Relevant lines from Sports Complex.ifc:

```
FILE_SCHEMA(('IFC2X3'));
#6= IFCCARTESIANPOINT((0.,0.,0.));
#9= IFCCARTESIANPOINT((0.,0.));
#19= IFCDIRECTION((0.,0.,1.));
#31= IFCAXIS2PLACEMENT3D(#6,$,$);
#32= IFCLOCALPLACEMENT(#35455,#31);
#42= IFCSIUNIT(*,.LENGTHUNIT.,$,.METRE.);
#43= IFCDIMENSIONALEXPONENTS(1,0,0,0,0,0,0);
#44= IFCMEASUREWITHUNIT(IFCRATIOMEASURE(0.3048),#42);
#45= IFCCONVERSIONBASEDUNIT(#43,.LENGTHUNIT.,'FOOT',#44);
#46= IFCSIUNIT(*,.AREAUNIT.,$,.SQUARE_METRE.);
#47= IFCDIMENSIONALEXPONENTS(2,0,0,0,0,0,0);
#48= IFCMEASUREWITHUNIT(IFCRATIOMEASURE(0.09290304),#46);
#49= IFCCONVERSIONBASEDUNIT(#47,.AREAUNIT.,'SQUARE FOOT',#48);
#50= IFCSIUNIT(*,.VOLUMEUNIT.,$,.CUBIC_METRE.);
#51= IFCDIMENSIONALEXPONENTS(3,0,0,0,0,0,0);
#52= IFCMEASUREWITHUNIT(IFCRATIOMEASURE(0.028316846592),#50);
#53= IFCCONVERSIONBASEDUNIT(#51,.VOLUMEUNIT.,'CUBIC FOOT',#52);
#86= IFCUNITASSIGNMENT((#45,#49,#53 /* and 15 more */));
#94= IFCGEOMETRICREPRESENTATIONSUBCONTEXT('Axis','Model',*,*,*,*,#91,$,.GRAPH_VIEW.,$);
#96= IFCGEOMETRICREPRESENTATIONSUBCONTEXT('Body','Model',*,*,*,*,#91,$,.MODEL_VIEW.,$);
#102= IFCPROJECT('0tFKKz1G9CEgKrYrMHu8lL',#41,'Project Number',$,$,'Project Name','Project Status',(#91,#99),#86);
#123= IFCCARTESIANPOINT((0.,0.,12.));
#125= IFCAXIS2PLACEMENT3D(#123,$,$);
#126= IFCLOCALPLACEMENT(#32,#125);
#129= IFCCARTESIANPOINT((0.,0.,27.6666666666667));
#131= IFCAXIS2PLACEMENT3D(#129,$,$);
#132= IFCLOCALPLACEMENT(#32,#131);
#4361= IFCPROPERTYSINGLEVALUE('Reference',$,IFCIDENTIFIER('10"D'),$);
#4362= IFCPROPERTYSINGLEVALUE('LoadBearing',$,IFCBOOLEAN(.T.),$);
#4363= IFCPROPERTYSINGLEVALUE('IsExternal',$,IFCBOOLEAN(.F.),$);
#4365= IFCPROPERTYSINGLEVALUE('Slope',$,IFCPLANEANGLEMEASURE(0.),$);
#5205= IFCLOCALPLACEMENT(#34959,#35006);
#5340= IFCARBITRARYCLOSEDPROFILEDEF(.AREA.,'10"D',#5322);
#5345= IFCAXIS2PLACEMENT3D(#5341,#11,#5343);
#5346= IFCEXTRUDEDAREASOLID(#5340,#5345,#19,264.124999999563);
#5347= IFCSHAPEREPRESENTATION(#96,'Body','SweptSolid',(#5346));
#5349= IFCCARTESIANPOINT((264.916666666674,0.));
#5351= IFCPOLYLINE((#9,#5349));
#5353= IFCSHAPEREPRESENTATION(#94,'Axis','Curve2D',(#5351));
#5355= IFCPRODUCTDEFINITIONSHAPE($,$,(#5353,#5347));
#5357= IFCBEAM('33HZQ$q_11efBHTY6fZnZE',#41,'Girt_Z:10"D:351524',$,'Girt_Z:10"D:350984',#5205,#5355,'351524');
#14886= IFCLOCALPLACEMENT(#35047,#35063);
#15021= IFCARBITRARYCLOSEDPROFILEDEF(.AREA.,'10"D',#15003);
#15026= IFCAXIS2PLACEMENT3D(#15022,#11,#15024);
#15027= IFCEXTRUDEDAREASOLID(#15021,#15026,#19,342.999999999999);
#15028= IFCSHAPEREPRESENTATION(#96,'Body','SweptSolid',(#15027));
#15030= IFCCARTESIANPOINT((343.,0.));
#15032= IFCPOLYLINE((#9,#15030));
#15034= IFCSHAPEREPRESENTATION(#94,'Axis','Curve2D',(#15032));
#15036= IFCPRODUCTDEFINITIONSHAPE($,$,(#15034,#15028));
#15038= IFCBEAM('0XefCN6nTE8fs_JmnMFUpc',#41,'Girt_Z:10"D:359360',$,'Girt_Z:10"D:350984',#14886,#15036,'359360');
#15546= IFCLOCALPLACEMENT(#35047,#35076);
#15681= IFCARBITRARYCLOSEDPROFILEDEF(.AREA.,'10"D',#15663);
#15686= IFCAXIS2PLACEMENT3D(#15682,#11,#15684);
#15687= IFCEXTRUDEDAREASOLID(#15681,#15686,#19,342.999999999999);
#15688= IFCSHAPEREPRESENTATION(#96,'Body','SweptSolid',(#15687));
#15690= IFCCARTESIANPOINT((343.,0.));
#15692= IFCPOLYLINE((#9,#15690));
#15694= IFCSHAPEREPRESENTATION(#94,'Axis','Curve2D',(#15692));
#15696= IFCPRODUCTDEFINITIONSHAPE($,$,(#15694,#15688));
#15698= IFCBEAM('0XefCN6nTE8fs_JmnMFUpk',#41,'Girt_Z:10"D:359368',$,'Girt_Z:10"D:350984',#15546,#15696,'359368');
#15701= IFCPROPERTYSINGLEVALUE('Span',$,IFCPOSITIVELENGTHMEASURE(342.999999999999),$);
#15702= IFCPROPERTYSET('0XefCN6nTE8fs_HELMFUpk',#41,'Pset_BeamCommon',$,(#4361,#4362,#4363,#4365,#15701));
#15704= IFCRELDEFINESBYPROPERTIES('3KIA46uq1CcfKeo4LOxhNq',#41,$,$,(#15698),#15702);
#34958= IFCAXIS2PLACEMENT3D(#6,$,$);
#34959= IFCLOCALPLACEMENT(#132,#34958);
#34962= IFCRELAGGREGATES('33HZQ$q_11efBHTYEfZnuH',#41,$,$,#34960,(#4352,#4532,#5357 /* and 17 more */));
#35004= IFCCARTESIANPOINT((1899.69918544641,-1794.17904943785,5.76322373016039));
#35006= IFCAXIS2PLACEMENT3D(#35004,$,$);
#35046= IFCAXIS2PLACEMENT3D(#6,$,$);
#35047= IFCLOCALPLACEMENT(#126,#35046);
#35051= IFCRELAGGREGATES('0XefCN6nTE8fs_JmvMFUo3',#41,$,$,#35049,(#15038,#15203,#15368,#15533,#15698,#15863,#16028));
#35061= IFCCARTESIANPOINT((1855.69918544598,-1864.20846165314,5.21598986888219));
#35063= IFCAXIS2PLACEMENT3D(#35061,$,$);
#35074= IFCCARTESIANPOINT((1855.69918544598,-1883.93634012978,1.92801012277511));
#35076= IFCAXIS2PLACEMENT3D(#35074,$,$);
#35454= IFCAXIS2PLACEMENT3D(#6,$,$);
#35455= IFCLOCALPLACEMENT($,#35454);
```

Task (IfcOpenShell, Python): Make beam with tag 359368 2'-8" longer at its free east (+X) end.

```python
import numpy as np
import ifcopenshell
import ifcopenshell.api.pset
import ifcopenshell.util.element
import ifcopenshell.util.representation
import ifcopenshell.util.unit

model = ifcopenshell.open("Sports Complex.ifc")
unit_scale = ifcopenshell.util.unit.calculate_unit_scale(model)

member = model.by_guid("0XefCN6nTE8fs_JmnMFUpk")
change = 32 * 0.0254 / unit_scale

# The extrusion runs towards the end named, so only its depth changes.
body = ifcopenshell.util.representation.get_representation(member, "Model", "Body")
solid = body.Items[0]
old_length = solid.Depth
solid.Depth += change

# Move the axis end point with it.
axis = next(r for r in member.Representation.Representations if r.RepresentationIdentifier == "Axis").Items[0]
start, end = (np.array(p.Coordinates) for p in axis.Points)
end = end + (end - start) / np.linalg.norm(end - start) * change
point = model.createIfcCartesianPoint(end.tolist())
axis.Points = [axis.Points[0], point]

# Update the stored length and volume.
pset = model.by_id(ifcopenshell.util.element.get_pset(member, "Pset_BeamCommon", should_inherit=False)["id"])
ifcopenshell.api.pset.edit_pset(model, pset=pset, properties={
    "Span": model.create_entity("IfcPositiveLengthMeasure", solid.Depth),
})

print(f"length {old_length:g} -> {solid.Depth:g}")

model.write("Sports Complex_rev.ifc")
```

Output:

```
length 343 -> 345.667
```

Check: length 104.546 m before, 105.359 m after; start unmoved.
